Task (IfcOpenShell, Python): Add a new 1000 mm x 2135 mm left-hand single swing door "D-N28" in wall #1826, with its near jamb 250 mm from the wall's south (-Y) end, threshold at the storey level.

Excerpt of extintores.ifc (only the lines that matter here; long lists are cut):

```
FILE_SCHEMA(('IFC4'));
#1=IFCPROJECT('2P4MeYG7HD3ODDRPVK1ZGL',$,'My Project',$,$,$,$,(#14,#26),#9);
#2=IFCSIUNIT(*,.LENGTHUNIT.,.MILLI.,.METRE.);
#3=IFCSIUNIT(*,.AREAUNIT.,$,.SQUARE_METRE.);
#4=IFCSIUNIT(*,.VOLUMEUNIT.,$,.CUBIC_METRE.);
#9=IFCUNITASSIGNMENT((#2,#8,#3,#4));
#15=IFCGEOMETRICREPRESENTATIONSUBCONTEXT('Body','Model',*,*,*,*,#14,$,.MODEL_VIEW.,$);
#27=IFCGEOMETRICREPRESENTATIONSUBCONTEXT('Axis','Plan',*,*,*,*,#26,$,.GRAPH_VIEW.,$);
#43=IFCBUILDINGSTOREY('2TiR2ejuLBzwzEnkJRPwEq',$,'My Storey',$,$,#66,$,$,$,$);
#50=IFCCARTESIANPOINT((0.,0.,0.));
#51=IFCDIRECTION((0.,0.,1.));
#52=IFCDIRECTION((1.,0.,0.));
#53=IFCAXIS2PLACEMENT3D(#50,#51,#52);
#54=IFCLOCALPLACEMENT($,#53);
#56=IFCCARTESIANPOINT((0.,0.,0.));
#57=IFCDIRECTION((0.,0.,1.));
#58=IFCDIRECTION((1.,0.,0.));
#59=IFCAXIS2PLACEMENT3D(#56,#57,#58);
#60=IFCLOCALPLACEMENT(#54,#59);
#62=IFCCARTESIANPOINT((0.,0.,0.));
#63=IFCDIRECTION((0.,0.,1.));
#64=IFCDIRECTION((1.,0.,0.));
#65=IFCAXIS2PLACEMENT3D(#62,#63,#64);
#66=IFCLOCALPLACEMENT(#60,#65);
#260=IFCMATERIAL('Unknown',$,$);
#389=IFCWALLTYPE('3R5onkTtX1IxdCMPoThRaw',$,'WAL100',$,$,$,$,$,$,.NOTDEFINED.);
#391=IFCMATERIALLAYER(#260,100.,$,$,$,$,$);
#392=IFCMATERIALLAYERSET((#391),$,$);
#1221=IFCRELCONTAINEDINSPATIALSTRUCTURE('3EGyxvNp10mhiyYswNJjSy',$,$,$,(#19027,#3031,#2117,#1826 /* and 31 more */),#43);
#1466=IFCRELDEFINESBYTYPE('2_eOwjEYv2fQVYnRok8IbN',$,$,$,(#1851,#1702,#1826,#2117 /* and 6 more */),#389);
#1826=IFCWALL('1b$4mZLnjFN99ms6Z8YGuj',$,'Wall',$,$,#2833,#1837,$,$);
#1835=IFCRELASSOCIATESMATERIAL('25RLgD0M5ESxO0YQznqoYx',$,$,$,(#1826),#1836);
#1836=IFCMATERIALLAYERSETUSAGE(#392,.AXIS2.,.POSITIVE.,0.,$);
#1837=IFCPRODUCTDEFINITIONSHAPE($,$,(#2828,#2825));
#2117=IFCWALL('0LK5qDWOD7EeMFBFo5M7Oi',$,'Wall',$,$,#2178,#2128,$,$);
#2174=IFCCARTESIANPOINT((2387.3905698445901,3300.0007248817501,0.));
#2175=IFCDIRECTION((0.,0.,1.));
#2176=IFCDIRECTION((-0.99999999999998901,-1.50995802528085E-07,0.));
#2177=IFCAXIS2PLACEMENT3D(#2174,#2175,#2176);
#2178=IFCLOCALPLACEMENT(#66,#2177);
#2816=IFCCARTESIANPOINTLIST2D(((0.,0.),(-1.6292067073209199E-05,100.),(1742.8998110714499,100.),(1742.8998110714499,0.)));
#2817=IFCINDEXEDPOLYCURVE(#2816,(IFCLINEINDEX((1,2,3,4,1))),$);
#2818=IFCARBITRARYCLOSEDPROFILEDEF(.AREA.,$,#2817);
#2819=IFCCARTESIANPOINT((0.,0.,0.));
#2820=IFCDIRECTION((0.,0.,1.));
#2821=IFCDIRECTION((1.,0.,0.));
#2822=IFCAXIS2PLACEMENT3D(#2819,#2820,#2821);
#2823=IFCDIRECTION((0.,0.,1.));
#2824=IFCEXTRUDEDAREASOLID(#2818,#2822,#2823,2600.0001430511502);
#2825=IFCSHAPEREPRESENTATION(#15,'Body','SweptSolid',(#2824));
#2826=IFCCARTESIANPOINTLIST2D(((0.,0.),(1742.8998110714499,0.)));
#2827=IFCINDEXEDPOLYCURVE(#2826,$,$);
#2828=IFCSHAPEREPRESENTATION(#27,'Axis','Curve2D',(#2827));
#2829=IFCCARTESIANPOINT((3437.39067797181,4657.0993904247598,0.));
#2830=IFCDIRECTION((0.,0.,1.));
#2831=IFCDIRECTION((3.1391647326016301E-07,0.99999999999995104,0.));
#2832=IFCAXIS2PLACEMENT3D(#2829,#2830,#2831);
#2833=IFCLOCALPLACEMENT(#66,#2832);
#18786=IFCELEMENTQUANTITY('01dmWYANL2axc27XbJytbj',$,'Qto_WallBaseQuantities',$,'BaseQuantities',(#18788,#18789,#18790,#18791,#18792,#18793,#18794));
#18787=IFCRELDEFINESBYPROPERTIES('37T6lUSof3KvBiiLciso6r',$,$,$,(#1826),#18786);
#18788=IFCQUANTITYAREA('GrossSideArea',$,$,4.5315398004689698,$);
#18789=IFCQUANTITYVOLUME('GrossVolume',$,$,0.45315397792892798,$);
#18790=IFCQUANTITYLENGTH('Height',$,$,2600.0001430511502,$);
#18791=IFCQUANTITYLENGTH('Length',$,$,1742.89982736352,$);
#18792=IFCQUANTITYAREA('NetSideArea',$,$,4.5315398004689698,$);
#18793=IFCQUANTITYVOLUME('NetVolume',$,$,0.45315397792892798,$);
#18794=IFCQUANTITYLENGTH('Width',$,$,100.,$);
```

```python
import numpy as np
import ifcopenshell
import ifcopenshell.api.feature
import ifcopenshell.api.geometry
import ifcopenshell.api.pset
import ifcopenshell.api.root
import ifcopenshell.api.spatial
import ifcopenshell.geom
import ifcopenshell.util.element
import ifcopenshell.util.placement
import ifcopenshell.util.representation
import ifcopenshell.util.shape
import ifcopenshell.util.unit

model = ifcopenshell.open("extintores.ifc")
unit_scale = ifcopenshell.util.unit.calculate_unit_scale(model)
area_scale = ifcopenshell.util.unit.calculate_unit_scale(model, "AREAUNIT")
volume_scale = ifcopenshell.util.unit.calculate_unit_scale(model, "VOLUMEUNIT")
settings = ifcopenshell.geom.settings()


def volume(element):
    """Net volume in cubic metres, openings subtracted."""
    shape = ifcopenshell.geom.create_shape(settings, element)
    return ifcopenshell.util.shape.get_volume(shape.geometry)


wall = model.by_guid("1b$4mZLnjFN99ms6Z8YGuj")
storey = ifcopenshell.util.element.get_container(wall, ifc_class="IfcBuildingStorey")
context = ifcopenshell.util.representation.get_context(model, "Model", "Body", "MODEL_VIEW")
before = volume(wall)

width, height, from_end, sill = 1, 2.135, 0.25, 0.0  # metres

# The wall runs along its own X axis, and the end named is its -X end.
wall_shape = ifcopenshell.geom.create_shape(settings, wall)
x, y, z = ifcopenshell.util.shape.get_vertices(wall_shape.geometry).T
start = x.min() + from_end
face, thickness = float(y.min()), float(y.max() - y.min())
wall_matrix = ifcopenshell.util.placement.get_local_placement(wall.ObjectPlacement)
level = ifcopenshell.util.placement.get_local_placement(storey.ObjectPlacement)[2, 3]


def in_wall(x, y):
    """Placement at x, y metres in the wall's axes, at sill height."""
    matrix = wall_matrix.copy()
    matrix[:, 3] = wall_matrix @ np.array([x / unit_scale, y / unit_scale, 0.0, 1.0])
    matrix[2, 3] = level + sill / unit_scale
    return matrix


# Opening: a box that overshoots both wall faces by 50 mm.
opening = ifcopenshell.api.root.create_entity(model, ifc_class="IfcOpeningElement", predefined_type="OPENING")
box = ifcopenshell.api.geometry.add_wall_representation(
    model, context=context, length=width, height=height, thickness=thickness + 0.1
)
ifcopenshell.api.geometry.assign_representation(model, product=opening, representation=box)
ifcopenshell.api.geometry.edit_object_placement(model, product=opening, matrix=in_wall(start, face - 0.05), is_si=False)
ifcopenshell.api.feature.add_feature(model, feature=opening, element=wall)

door = ifcopenshell.api.root.create_entity(model, ifc_class="IfcDoor", name="D-N28", predefined_type="DOOR")
door.OverallWidth, door.OverallHeight = width / unit_scale, height / unit_scale
door.OperationType = "SINGLE_SWING_LEFT"
body = ifcopenshell.api.geometry.add_door_representation(
    model,
    context=context,
    overall_width=door.OverallWidth,
    overall_height=door.OverallHeight,
    operation_type="SINGLE_SWING_LEFT",
    lining_properties={"LiningDepth": thickness / unit_scale, "ThresholdDepth": thickness / unit_scale},
)
ifcopenshell.api.geometry.assign_representation(model, product=door, representation=body)
ifcopenshell.api.spatial.assign_container(model, products=[door], relating_structure=storey)
ifcopenshell.api.feature.add_filling(model, opening=opening, element=door)

# The lining spans the wall, so the door starts at the wall face.
ifcopenshell.api.geometry.edit_object_placement(model, product=door, matrix=in_wall(start, face), is_si=False)

after = volume(wall)

# Update the wall's stored quantities.
qto = model.by_id(ifcopenshell.util.element.get_pset(wall, "Qto_WallBaseQuantities", should_inherit=False)["id"])
ifcopenshell.api.pset.edit_qto(model, qto=qto, properties={
    "NetSideArea": after / thickness / area_scale,
    "NetVolume": after / volume_scale,
})

print(f"wall volume {before:.3f} -> {after:.3f} m3")

model.write("extintores_v2.ifc")
```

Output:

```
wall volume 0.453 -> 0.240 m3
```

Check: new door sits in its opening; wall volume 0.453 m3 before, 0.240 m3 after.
